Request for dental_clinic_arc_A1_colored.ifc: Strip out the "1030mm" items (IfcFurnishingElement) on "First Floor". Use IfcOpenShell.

First a look at what the model holds.

```python
import ifcopenshell
import ifcopenshell.util.element

model = ifcopenshell.open("dental_clinic_arc_A1_colored.ifc")
print(model.schema)
storey = next(s for s in model.by_type("IfcBuildingStorey") if s.Name == "First Floor")
furniture = [e for e in ifcopenshell.util.element.get_decomposition(storey) if e.is_a("IfcFurnishingElement")]
seen = {}
for e in furniture:
    element_type = ifcopenshell.util.element.get_type(e)
    name = element_type.Name if element_type not in (None, e) else None
    seen[name] = seen.get(name, 0) + 1
for name, count in sorted(seen.items(), key=str):
    print(count, "x", name)
```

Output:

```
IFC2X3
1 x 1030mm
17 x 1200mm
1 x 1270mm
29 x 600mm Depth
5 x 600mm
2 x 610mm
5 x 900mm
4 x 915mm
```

```python
import ifcopenshell
import ifcopenshell.api.root
import ifcopenshell.util.element

model = ifcopenshell.open("dental_clinic_arc_A1_colored.ifc")

storey = next(s for s in model.by_type("IfcBuildingStorey") if s.Name == "First Floor")
furniture = [e for e in ifcopenshell.util.element.get_decomposition(storey) if e.is_a("IfcFurnishingElement")]
targets = [e for e in furniture if (t := ifcopenshell.util.element.get_type(e)) not in (None, e) and t.Name == "1030mm"]

for e in targets:
    ifcopenshell.api.root.remove_product(model, product=e)
print(len(targets), "removed")

model.write("dental_clinic_arc_A1_colored_edited.ifc")
```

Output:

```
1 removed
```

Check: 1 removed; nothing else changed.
